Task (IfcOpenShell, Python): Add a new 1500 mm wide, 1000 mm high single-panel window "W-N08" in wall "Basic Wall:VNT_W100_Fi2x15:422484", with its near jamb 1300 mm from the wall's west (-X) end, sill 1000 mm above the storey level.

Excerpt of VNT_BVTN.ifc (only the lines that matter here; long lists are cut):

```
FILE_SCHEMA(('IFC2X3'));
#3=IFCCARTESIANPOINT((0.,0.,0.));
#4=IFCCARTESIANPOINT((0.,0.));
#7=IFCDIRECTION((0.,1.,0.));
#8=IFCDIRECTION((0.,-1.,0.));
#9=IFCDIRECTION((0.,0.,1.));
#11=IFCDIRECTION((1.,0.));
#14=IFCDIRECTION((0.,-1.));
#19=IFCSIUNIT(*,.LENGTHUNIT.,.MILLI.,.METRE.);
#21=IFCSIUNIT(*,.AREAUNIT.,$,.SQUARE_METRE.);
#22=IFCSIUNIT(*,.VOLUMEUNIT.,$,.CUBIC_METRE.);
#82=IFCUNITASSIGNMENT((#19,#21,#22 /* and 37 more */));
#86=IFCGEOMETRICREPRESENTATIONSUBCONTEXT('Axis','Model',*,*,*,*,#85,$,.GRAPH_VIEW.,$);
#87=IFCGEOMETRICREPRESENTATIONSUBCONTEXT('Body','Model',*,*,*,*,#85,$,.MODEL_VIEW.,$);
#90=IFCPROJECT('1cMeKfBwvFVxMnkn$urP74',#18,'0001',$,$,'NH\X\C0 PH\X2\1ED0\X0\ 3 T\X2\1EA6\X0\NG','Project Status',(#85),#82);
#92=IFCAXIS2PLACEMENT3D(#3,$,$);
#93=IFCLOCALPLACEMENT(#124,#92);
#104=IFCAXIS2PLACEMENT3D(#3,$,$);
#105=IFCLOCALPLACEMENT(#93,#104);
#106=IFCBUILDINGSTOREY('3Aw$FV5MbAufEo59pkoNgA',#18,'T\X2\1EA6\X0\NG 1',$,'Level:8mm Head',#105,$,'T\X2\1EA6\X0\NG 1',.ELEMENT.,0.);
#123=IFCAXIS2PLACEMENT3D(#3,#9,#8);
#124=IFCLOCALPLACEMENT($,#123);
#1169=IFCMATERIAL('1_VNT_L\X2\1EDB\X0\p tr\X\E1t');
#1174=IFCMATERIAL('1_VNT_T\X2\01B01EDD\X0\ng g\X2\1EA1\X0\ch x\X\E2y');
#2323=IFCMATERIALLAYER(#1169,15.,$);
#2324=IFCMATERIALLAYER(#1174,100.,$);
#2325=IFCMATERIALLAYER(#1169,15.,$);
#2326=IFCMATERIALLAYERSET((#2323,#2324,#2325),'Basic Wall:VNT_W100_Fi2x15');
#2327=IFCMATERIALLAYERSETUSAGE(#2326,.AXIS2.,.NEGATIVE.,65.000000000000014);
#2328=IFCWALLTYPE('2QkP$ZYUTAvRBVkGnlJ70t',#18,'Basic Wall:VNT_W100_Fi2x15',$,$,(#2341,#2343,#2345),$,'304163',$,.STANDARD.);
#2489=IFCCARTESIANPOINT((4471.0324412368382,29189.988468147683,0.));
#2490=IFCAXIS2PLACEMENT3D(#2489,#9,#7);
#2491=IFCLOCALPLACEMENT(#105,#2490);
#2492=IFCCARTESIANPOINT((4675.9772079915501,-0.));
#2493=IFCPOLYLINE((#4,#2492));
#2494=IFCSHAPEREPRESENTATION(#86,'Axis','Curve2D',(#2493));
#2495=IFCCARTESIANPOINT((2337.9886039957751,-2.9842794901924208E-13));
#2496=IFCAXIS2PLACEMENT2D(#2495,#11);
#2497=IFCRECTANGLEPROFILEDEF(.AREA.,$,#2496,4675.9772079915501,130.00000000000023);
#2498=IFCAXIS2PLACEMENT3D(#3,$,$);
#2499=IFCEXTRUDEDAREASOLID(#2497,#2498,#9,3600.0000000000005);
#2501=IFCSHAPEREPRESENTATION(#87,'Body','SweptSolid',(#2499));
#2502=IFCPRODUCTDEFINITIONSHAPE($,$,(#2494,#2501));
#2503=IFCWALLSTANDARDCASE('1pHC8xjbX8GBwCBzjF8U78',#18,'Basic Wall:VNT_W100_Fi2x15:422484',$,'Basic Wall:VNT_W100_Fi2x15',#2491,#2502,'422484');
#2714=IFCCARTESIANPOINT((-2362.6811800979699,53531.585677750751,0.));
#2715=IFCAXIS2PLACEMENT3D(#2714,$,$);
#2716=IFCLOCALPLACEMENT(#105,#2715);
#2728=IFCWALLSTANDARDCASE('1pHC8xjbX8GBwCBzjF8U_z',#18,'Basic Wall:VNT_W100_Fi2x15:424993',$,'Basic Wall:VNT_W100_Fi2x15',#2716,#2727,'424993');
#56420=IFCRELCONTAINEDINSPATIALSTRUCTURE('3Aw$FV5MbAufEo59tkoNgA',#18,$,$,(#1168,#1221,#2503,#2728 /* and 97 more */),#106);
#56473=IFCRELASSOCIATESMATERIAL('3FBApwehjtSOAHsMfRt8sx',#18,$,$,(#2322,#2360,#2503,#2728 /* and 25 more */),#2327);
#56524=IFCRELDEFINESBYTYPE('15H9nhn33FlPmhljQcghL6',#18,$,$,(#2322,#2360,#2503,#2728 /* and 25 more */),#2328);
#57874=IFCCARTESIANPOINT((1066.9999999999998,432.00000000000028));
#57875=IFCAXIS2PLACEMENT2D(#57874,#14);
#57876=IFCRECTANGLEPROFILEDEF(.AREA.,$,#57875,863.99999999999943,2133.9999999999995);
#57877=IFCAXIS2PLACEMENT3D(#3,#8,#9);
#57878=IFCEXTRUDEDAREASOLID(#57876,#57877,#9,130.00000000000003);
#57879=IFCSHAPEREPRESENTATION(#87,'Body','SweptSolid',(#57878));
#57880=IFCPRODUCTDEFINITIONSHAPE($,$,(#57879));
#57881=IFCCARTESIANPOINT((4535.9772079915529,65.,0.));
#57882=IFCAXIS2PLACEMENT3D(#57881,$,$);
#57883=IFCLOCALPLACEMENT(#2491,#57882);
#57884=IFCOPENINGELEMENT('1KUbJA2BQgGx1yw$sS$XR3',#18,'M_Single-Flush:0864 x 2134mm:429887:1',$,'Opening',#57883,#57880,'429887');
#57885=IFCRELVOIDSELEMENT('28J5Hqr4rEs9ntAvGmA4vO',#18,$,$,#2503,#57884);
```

```python
import numpy as np
import ifcopenshell
import ifcopenshell.api.feature
import ifcopenshell.api.geometry
import ifcopenshell.api.root
import ifcopenshell.api.spatial
import ifcopenshell.api.type
import ifcopenshell.geom
import ifcopenshell.util.element
import ifcopenshell.util.placement
import ifcopenshell.util.representation
import ifcopenshell.util.shape
import ifcopenshell.util.unit

model = ifcopenshell.open("VNT_BVTN.ifc")
unit_scale = ifcopenshell.util.unit.calculate_unit_scale(model)
settings = ifcopenshell.geom.settings()


def volume(element):
    """Net volume in cubic metres, openings subtracted."""
    shape = ifcopenshell.geom.create_shape(settings, element)
    return ifcopenshell.util.shape.get_volume(shape.geometry)


wall = model.by_guid("1pHC8xjbX8GBwCBzjF8U78")
storey = ifcopenshell.util.element.get_container(wall, ifc_class="IfcBuildingStorey")
context = ifcopenshell.util.representation.get_context(model, "Model", "Body", "MODEL_VIEW")
before = volume(wall)

width, height, from_end, sill = 1.5, 1, 1.3, 1  # metres

# The wall runs along its own X axis, and the end named is its -X end.
wall_shape = ifcopenshell.geom.create_shape(settings, wall)
x, y, z = ifcopenshell.util.shape.get_vertices(wall_shape.geometry).T
start = x.min() + from_end
face, thickness = float(y.min()), float(y.max() - y.min())
wall_matrix = ifcopenshell.util.placement.get_local_placement(wall.ObjectPlacement)
level = ifcopenshell.util.placement.get_local_placement(storey.ObjectPlacement)[2, 3]


def in_wall(x, y):
    """Placement at x, y metres in the wall's axes, at sill height."""
    matrix = wall_matrix.copy()
    matrix[:, 3] = wall_matrix @ np.array([x / unit_scale, y / unit_scale, 0.0, 1.0])
    matrix[2, 3] = level + sill / unit_scale
    return matrix


# Opening: a box that overshoots both wall faces by 50 mm.
opening = ifcopenshell.api.root.create_entity(model, ifc_class="IfcOpeningElement")
box = ifcopenshell.api.geometry.add_wall_representation(
    model, context=context, length=width, height=height, thickness=thickness + 0.1
)
ifcopenshell.api.geometry.assign_representation(model, product=opening, representation=box)
ifcopenshell.api.geometry.edit_object_placement(model, product=opening, matrix=in_wall(start, face - 0.05), is_si=False)
ifcopenshell.api.feature.add_feature(model, feature=opening, element=wall)

window = ifcopenshell.api.root.create_entity(model, ifc_class="IfcWindow", name="W-N08")
window.OverallWidth, window.OverallHeight = width / unit_scale, height / unit_scale
body = ifcopenshell.api.geometry.add_window_representation(
    model,
    context=context,
    overall_width=window.OverallWidth,
    overall_height=window.OverallHeight,
    partition_type="SINGLE_PANEL",
)
ifcopenshell.api.geometry.assign_representation(model, product=window, representation=body)
ifcopenshell.api.spatial.assign_container(model, products=[window], relating_structure=storey)
fills = ifcopenshell.api.feature.add_filling(model, opening=opening, element=window)
fills.OwnerHistory = window.OwnerHistory  # required in IFC2X3

# IFC2X3 keeps the operation on the window style.
style = ifcopenshell.api.root.create_entity(model, ifc_class="IfcWindowStyle", name="W-N08")
style.OperationType, style.ConstructionType = "SINGLE_PANEL", "NOTDEFINED"
style.ParameterTakesPrecedence = style.Sizeable = False
ifcopenshell.api.type.assign_type(model, related_objects=[window], relating_type=style)

# Centre the window in the wall's thickness.
ifcopenshell.api.geometry.edit_object_placement(model, product=window, matrix=in_wall(start, face), is_si=False)
window_shape = ifcopenshell.geom.create_shape(settings, window)
depth = ifcopenshell.util.shape.get_vertices(window_shape.geometry)[:, 1]
offset = face + thickness / 2 - (depth.min() + depth.max()) / 2
ifcopenshell.api.geometry.edit_object_placement(model, product=window, matrix=in_wall(start, offset), is_si=False)

after = volume(wall)

print(f"wall volume {before:.3f} -> {after:.3f} m3")

model.write("VNT_BVTN-out.ifc")
```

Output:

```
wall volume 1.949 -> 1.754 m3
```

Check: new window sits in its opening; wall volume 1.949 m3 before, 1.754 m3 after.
